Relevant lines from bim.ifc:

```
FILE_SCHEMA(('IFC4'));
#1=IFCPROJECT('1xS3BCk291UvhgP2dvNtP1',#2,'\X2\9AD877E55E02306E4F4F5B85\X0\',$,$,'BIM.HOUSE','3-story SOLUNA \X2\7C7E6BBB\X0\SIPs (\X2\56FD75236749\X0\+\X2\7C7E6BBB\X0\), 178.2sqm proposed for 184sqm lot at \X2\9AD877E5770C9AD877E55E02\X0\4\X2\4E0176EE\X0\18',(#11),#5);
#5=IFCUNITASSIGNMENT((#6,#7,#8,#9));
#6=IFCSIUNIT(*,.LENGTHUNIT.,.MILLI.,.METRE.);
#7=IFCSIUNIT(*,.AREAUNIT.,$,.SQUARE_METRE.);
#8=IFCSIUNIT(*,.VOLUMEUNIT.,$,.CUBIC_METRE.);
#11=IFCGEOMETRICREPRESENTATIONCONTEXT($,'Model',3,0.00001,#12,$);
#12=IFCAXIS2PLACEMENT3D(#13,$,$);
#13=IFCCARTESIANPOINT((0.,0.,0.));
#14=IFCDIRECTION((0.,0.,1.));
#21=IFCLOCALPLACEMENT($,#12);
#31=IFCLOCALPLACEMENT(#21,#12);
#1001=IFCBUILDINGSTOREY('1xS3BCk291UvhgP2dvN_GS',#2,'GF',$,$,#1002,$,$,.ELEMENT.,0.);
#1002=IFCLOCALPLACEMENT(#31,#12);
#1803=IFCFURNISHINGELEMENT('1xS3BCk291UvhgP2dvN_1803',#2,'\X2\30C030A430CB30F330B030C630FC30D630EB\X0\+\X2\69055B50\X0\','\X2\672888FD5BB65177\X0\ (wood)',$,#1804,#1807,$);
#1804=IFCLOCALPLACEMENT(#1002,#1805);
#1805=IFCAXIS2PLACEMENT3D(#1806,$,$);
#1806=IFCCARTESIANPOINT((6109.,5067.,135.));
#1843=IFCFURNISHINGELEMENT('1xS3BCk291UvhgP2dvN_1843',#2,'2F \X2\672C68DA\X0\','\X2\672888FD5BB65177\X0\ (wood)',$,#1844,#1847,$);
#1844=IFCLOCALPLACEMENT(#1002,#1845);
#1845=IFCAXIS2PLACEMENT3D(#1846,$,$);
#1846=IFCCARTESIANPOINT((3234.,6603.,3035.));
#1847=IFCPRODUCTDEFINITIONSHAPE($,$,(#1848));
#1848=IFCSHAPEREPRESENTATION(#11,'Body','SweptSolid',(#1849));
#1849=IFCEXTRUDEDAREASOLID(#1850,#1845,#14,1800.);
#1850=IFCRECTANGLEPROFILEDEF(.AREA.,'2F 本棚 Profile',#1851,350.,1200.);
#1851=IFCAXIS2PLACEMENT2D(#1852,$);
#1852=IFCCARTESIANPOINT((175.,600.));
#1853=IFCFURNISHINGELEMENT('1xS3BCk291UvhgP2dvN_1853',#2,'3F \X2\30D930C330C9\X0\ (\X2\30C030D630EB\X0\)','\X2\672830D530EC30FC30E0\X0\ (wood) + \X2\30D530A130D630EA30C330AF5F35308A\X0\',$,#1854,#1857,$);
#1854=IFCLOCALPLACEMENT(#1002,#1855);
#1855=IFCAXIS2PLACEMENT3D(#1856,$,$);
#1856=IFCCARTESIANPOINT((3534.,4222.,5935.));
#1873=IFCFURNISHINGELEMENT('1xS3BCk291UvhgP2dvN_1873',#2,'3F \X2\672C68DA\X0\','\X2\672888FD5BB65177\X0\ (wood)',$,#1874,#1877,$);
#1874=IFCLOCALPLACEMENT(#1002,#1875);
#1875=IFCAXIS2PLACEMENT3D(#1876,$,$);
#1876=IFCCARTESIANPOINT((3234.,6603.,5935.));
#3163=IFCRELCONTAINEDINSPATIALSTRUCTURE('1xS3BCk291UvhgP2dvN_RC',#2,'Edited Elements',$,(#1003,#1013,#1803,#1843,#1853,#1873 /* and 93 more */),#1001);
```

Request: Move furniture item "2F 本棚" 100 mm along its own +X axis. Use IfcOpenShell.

```python
import ifcopenshell
import ifcopenshell.api.geometry
import ifcopenshell.util.placement
import ifcopenshell.util.unit

model = ifcopenshell.open("bim.ifc")
unit_scale = ifcopenshell.util.unit.calculate_unit_scale(model)

item = model.by_guid("1xS3BCk291UvhgP2dvN_1843")
matrix = ifcopenshell.util.placement.get_local_placement(item.ObjectPlacement)
matrix[:3, 3] += matrix[:3, 0] * 0.1 / unit_scale
ifcopenshell.api.geometry.edit_object_placement(model, product=item, matrix=matrix, is_si=False)

print(ifcopenshell.util.placement.get_local_placement(item.ObjectPlacement).round(3) + 0.0)

model.write("bim_v2.ifc")
```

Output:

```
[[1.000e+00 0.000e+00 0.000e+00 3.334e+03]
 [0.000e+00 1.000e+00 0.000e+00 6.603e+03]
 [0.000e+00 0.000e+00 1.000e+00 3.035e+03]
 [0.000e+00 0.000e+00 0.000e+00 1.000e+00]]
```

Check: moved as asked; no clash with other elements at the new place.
